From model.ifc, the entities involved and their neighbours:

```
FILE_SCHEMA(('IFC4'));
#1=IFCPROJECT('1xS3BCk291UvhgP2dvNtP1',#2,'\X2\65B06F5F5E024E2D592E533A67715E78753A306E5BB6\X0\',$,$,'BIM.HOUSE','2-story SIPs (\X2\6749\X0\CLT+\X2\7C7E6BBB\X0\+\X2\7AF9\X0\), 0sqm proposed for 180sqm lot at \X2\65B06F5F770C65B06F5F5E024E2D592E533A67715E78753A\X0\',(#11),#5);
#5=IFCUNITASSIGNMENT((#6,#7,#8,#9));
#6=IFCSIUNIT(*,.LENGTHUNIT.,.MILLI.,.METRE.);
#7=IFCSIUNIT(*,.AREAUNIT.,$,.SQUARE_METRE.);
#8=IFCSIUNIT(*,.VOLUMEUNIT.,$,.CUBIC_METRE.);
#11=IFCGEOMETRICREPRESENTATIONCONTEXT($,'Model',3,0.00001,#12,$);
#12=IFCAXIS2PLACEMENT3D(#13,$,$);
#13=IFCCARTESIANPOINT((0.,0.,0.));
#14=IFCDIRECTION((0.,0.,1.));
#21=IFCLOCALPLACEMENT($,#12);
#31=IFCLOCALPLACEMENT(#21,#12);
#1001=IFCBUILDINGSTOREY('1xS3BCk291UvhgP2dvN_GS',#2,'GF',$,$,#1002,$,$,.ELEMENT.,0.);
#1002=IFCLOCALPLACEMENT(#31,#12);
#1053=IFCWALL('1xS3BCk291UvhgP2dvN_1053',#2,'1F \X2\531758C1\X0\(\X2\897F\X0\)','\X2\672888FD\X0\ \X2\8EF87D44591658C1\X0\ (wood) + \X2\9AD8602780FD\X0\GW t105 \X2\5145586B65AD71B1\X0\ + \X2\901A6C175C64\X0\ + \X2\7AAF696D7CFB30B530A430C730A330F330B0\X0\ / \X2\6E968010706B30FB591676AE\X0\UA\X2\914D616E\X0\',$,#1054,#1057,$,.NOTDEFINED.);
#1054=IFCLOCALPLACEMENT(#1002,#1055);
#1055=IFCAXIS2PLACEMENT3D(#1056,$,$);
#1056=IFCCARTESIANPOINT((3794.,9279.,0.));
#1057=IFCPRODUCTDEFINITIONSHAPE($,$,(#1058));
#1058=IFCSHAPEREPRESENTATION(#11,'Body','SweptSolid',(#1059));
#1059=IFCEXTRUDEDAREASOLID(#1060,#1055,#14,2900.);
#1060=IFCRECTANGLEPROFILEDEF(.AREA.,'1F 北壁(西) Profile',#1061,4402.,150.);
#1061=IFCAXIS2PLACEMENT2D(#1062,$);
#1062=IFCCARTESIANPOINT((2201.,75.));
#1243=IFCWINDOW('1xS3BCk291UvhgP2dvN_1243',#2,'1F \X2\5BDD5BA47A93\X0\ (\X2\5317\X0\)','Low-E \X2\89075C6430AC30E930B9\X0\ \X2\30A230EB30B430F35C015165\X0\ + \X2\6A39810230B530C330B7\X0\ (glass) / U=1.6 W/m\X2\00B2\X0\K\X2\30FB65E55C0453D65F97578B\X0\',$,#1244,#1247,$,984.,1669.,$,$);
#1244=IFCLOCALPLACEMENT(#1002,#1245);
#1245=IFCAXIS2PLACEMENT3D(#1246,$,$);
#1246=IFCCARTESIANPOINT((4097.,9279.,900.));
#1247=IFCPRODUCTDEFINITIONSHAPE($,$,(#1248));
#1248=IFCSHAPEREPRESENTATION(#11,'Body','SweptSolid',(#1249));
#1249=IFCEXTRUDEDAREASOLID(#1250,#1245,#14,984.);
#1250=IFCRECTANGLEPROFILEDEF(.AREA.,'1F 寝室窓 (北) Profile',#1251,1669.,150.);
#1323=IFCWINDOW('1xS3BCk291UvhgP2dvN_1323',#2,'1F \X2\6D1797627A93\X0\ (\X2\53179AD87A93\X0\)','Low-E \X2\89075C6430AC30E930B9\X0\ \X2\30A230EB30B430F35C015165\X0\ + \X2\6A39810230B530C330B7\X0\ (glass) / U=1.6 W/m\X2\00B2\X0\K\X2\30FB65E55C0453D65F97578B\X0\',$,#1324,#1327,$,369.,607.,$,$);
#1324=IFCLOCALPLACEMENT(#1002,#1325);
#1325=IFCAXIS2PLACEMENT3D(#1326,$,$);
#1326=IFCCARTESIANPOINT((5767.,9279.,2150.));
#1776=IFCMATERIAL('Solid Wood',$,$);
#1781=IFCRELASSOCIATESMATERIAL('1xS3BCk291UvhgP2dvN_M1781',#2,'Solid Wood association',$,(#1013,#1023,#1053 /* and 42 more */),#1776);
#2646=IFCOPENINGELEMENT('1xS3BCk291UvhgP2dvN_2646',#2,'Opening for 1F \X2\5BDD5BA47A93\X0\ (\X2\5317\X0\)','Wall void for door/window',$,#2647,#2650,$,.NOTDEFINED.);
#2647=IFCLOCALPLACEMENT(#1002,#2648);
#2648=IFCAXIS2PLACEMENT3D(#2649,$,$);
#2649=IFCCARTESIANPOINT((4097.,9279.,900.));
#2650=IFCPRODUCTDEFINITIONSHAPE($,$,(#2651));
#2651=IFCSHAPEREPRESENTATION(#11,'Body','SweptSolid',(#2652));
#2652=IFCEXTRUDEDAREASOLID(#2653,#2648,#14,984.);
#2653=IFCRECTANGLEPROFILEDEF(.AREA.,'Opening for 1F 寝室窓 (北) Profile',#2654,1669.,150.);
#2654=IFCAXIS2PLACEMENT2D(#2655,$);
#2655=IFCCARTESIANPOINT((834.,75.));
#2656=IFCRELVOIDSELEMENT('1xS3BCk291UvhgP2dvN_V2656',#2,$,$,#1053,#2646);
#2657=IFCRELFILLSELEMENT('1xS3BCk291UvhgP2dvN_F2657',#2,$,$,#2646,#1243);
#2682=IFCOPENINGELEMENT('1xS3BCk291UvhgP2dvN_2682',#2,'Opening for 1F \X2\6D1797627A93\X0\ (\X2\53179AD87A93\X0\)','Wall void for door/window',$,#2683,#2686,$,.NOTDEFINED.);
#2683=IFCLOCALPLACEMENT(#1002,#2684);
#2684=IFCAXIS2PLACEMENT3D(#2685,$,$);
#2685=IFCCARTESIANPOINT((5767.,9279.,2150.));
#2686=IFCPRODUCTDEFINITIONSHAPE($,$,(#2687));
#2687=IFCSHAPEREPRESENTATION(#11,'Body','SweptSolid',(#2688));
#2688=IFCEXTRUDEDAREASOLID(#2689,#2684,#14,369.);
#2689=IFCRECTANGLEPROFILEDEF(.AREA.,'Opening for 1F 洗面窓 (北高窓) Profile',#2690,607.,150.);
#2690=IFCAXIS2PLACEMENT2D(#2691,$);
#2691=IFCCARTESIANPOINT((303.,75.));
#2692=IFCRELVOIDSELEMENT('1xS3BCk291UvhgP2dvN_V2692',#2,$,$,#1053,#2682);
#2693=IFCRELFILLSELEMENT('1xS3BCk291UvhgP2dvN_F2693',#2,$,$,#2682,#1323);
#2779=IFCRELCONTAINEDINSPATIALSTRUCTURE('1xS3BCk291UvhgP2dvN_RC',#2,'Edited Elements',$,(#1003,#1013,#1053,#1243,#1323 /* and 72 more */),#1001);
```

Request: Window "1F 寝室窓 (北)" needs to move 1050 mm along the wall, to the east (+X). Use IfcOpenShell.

```python
import ifcopenshell
import ifcopenshell.api.geometry
import ifcopenshell.util.placement
import ifcopenshell.util.unit

model = ifcopenshell.open("model.ifc")
unit_scale = ifcopenshell.util.unit.calculate_unit_scale(model)

window = model.by_guid("1xS3BCk291UvhgP2dvN_1243")
opening = window.FillsVoids[0].RelatingOpeningElement
wall = opening.VoidsElements[0].RelatingBuildingElement

wall_matrix = ifcopenshell.util.placement.get_local_placement(wall.ObjectPlacement)
shift = wall_matrix[:3, 0] * 1.05 / unit_scale
before = ifcopenshell.util.placement.get_local_placement(window.ObjectPlacement)[:3, 3].copy()

# The window is not placed relative to its opening, so move both.
for product in (opening, window):
    matrix = ifcopenshell.util.placement.get_local_placement(product.ObjectPlacement)
    matrix[:3, 3] += shift
    ifcopenshell.api.geometry.edit_object_placement(model, product=product, matrix=matrix, is_si=False)

after = ifcopenshell.util.placement.get_local_placement(window.ObjectPlacement)[:3, 3]
print("window moved by", (after - before).round(3) + 0.0)

model.write("model_v2.ifc")
```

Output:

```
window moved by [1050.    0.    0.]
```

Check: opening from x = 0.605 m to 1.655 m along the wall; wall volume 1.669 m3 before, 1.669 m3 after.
